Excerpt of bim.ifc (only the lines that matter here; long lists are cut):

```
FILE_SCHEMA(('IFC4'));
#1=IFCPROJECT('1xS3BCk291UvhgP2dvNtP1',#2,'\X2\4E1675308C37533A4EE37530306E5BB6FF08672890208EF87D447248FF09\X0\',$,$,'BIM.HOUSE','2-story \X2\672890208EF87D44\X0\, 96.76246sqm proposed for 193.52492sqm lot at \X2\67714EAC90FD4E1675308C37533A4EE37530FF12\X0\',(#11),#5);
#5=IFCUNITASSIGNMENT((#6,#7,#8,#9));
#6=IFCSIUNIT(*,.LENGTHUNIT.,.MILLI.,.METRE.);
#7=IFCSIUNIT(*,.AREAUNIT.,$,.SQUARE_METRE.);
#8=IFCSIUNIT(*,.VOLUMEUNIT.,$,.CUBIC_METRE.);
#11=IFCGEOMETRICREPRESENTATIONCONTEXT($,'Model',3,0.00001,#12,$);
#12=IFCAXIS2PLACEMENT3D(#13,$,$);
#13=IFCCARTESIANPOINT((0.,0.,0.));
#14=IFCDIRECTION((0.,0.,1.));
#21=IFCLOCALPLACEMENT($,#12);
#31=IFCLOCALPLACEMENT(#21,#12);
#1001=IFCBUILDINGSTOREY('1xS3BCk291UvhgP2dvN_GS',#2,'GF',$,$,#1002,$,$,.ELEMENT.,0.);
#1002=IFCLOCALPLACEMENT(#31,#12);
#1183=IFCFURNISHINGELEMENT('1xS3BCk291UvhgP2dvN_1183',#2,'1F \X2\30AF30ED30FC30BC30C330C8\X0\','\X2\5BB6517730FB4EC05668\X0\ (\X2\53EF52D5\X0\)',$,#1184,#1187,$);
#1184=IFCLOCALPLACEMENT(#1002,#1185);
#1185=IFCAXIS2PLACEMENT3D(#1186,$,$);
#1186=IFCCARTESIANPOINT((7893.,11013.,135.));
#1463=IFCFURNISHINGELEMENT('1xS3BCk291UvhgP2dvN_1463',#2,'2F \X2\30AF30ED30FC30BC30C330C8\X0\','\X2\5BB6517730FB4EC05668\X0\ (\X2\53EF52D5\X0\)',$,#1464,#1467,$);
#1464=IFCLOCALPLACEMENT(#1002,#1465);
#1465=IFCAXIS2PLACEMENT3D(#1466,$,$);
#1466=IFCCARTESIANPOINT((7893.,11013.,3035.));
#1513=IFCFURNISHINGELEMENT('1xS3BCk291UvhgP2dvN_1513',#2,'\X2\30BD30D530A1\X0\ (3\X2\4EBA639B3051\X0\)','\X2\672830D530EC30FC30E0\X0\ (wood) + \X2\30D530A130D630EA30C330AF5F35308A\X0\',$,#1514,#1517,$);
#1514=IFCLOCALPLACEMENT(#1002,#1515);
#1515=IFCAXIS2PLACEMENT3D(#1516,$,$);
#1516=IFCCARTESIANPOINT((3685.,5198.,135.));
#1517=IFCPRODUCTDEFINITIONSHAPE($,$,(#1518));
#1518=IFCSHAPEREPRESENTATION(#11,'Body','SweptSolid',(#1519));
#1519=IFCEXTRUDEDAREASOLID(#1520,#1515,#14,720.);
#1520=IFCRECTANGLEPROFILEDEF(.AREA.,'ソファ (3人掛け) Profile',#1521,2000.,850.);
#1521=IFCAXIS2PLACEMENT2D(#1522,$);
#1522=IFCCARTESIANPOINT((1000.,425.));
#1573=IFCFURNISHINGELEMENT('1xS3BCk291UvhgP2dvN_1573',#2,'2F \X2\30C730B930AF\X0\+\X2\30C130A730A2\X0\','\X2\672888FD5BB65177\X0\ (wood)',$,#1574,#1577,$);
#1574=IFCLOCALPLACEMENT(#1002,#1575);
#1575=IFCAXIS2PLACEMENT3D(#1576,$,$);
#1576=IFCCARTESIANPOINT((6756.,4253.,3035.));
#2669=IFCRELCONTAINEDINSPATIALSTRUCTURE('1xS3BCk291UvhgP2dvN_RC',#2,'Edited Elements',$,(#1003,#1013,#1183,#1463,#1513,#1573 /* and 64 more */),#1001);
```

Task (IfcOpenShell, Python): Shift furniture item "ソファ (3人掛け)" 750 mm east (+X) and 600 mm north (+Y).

```python
import ifcopenshell
import ifcopenshell.api.geometry
import ifcopenshell.util.placement
import ifcopenshell.util.unit

model = ifcopenshell.open("bim.ifc")
unit_scale = ifcopenshell.util.unit.calculate_unit_scale(model)

item = model.by_guid("1xS3BCk291UvhgP2dvN_1513")
matrix = ifcopenshell.util.placement.get_local_placement(item.ObjectPlacement)
matrix[0, 3] += 0.75 / unit_scale
matrix[1, 3] += 0.6 / unit_scale
ifcopenshell.api.geometry.edit_object_placement(model, product=item, matrix=matrix, is_si=False)

print(ifcopenshell.util.placement.get_local_placement(item.ObjectPlacement).round(3) + 0.0)

model.write("bim_edited.ifc")
```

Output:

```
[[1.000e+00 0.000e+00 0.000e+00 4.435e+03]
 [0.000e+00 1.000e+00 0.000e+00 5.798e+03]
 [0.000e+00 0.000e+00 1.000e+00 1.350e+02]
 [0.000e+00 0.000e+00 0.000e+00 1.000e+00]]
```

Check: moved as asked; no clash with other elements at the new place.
